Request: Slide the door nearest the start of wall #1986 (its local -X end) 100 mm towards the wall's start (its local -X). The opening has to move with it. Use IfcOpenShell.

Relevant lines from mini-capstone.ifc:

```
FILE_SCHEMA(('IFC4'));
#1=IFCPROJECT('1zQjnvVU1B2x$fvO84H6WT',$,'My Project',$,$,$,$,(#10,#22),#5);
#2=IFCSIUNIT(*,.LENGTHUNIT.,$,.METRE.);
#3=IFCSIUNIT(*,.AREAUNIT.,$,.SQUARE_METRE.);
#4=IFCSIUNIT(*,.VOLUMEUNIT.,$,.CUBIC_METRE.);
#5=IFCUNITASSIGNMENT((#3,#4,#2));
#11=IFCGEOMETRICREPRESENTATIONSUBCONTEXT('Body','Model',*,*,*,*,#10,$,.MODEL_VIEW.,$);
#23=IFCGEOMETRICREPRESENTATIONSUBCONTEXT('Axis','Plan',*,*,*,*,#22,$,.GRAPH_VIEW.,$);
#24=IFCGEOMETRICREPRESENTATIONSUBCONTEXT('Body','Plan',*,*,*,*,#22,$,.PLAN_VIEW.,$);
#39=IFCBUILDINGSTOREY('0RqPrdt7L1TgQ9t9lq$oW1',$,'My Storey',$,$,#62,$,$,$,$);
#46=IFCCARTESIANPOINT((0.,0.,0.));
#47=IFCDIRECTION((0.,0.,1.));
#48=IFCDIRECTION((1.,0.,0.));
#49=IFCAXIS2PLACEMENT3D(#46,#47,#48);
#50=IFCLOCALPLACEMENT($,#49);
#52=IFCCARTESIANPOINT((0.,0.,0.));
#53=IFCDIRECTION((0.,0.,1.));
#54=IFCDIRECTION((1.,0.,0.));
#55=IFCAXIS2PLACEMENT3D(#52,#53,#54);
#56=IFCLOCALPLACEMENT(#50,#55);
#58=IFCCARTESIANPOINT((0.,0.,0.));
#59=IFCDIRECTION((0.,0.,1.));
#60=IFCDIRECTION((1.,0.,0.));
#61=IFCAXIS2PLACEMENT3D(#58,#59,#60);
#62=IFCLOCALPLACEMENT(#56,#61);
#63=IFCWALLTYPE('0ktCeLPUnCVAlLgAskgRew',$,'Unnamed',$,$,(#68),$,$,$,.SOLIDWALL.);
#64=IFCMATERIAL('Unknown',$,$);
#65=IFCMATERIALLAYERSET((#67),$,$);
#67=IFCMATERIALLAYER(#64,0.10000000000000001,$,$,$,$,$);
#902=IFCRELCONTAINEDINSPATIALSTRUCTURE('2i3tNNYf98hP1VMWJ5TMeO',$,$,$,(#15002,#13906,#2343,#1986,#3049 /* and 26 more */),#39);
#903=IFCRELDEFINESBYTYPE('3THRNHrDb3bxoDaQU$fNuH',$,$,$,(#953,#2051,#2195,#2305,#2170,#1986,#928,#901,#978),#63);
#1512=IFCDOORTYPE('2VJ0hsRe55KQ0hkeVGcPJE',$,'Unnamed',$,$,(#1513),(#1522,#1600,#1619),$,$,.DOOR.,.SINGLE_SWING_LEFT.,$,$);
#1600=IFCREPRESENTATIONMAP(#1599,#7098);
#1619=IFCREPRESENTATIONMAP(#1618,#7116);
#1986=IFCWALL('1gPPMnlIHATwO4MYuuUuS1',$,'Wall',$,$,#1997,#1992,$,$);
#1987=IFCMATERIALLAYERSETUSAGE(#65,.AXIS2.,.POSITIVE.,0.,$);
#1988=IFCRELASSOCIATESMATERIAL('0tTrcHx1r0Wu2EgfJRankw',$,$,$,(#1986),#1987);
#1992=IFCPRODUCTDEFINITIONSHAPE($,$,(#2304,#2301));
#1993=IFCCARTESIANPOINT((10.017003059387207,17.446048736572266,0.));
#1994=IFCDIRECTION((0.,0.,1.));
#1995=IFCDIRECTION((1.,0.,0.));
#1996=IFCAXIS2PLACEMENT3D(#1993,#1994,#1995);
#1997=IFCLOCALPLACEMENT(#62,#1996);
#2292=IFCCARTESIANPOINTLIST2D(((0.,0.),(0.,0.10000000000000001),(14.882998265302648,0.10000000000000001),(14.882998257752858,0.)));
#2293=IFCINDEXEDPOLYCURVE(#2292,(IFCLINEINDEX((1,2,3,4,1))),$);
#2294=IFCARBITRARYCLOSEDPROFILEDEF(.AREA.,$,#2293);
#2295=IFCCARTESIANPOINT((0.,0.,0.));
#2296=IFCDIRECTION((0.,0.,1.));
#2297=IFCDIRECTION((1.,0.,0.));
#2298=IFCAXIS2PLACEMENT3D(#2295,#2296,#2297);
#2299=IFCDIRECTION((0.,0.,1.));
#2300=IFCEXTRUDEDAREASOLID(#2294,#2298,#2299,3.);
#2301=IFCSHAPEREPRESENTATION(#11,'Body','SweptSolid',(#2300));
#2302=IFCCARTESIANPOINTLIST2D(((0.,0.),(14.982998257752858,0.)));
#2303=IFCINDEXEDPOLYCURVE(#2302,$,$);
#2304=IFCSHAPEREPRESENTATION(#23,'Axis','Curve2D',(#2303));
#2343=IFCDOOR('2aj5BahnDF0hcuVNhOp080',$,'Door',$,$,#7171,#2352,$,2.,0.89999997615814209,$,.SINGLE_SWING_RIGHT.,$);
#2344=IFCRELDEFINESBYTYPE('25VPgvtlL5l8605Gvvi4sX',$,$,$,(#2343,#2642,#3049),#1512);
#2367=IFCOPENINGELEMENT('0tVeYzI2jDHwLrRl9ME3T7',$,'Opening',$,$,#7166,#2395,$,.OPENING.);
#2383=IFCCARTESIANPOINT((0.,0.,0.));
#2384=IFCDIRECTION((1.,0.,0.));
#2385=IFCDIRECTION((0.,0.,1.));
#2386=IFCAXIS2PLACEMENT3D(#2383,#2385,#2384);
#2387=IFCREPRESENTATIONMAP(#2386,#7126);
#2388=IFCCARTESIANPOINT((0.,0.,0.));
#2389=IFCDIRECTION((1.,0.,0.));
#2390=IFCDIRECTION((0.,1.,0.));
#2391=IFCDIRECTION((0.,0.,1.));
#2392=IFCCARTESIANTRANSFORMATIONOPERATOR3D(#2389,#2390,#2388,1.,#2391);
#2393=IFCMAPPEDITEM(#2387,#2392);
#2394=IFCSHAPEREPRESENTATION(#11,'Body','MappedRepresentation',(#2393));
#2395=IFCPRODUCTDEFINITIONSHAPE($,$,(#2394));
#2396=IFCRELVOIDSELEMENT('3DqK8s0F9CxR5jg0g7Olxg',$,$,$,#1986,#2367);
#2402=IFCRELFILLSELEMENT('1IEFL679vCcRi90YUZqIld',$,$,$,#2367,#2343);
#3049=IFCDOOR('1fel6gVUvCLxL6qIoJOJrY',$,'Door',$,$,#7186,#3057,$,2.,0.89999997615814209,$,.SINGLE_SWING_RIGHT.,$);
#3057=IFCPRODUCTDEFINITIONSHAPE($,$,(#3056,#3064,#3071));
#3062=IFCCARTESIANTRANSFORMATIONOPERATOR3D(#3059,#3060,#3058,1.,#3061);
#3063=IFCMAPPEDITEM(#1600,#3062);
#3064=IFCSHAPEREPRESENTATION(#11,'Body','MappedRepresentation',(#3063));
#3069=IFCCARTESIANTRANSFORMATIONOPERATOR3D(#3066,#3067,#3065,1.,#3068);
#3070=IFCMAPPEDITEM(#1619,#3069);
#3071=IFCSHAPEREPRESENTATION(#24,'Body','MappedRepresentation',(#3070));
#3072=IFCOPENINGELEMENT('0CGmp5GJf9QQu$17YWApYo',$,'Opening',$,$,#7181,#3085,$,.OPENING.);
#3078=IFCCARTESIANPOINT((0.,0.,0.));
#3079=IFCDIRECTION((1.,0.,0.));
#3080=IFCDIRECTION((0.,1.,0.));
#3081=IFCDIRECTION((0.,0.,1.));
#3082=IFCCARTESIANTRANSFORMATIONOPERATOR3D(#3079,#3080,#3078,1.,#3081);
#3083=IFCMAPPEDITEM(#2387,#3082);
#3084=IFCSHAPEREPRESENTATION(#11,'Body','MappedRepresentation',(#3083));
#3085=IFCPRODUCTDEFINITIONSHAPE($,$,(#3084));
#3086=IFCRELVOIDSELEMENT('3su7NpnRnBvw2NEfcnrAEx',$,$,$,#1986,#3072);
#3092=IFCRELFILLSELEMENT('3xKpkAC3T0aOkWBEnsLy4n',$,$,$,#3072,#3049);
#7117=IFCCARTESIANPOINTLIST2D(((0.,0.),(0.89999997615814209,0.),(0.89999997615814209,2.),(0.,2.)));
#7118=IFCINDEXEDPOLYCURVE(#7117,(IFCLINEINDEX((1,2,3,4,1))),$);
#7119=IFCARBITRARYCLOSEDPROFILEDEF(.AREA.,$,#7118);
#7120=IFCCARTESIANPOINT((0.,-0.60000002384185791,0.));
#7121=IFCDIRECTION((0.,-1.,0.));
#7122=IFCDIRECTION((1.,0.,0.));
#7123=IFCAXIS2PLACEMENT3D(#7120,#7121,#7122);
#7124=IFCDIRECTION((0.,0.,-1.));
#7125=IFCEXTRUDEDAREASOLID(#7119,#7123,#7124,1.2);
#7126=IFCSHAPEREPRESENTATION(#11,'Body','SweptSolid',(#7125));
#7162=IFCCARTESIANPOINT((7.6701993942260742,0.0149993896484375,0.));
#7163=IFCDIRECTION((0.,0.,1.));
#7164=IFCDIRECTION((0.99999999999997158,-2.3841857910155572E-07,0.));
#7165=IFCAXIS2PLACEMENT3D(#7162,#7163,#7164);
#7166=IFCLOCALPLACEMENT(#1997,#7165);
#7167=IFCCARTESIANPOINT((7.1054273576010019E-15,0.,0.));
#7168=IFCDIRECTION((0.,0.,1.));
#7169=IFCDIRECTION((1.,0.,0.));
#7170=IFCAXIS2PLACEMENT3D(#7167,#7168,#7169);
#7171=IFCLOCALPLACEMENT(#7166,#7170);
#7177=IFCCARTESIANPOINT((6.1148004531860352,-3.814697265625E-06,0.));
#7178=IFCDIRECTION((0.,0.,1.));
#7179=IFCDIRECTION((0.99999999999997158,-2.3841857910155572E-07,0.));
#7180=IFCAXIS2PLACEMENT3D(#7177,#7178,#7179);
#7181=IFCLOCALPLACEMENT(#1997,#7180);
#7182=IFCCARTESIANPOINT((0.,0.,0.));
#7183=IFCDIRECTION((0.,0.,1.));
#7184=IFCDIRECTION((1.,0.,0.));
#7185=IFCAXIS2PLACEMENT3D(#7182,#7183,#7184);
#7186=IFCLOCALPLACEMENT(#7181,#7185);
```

```python
import ifcopenshell
import ifcopenshell.api.geometry
import ifcopenshell.util.placement
import ifcopenshell.util.unit

model = ifcopenshell.open("mini-capstone.ifc")
unit_scale = ifcopenshell.util.unit.calculate_unit_scale(model)

door = model.by_id(3049)
opening = door.FillsVoids[0].RelatingOpeningElement
wall = opening.VoidsElements[0].RelatingBuildingElement

wall_matrix = ifcopenshell.util.placement.get_local_placement(wall.ObjectPlacement)
shift = wall_matrix[:3, 0] * -0.1 / unit_scale
before = ifcopenshell.util.placement.get_local_placement(door.ObjectPlacement)[:3, 3].copy()

# The door is placed relative to its opening, so it follows when the opening moves.
matrix = ifcopenshell.util.placement.get_local_placement(opening.ObjectPlacement)
matrix[:3, 3] += shift
ifcopenshell.api.geometry.edit_object_placement(
    model, product=opening, matrix=matrix, is_si=False, should_transform_children=True
)

after = ifcopenshell.util.placement.get_local_placement(door.ObjectPlacement)[:3, 3]
print("door moved by", (after - before).round(3) + 0.0)

model.write("mini-capstone_rev.ifc")
```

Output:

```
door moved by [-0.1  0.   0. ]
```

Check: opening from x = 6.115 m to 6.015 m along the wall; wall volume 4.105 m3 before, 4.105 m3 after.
